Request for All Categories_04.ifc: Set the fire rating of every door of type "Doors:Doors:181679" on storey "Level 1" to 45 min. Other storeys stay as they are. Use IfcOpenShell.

First a look at what the model holds.

```python
import ifcopenshell
import ifcopenshell.util.element

model = ifcopenshell.open("All Categories_04.ifc")
print(model.schema)
storey = next(s for s in model.by_type("IfcBuildingStorey") if s.Name == "Level 1")
doors = [e for e in ifcopenshell.util.element.get_decomposition(storey) if e.is_a("IfcDoor")]
seen = {}
for e in doors:
    element_type = ifcopenshell.util.element.get_type(e)
    key = (element_type.Name if element_type != e and element_type else None, ifcopenshell.util.element.get_pset(e, "Pset_DoorCommon", "FireRating"))
    seen[key] = seen.get(key, 0) + 1
for (name, value), count in sorted(seen.items(), key=str):
    print(count, "x", name, "|", value)
```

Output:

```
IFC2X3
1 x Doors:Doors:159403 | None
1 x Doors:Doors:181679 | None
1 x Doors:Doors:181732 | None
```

```python
import ifcopenshell
import ifcopenshell.api.pset
import ifcopenshell.util.element

model = ifcopenshell.open("All Categories_04.ifc")

storey = next(s for s in model.by_type("IfcBuildingStorey") if s.Name == "Level 1")
doors = [e for e in ifcopenshell.util.element.get_decomposition(storey) if e.is_a("IfcDoor")]

count = 0
for e in doors:
    element_type = ifcopenshell.util.element.get_type(e)
    if element_type in (None, e) or element_type.Name != "Doors:Doors:181679":
        continue
    # add_pset returns the element's existing set when there is one.
    pset = ifcopenshell.api.pset.add_pset(model, product=e, name="Pset_DoorCommon")
    ifcopenshell.api.pset.edit_pset(model, pset=pset, properties={"FireRating": "45 min"})
    count += 1

print(count, "doors updated")

model.write("All Categories_04_edited.ifc")
```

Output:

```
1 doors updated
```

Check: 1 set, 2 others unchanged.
